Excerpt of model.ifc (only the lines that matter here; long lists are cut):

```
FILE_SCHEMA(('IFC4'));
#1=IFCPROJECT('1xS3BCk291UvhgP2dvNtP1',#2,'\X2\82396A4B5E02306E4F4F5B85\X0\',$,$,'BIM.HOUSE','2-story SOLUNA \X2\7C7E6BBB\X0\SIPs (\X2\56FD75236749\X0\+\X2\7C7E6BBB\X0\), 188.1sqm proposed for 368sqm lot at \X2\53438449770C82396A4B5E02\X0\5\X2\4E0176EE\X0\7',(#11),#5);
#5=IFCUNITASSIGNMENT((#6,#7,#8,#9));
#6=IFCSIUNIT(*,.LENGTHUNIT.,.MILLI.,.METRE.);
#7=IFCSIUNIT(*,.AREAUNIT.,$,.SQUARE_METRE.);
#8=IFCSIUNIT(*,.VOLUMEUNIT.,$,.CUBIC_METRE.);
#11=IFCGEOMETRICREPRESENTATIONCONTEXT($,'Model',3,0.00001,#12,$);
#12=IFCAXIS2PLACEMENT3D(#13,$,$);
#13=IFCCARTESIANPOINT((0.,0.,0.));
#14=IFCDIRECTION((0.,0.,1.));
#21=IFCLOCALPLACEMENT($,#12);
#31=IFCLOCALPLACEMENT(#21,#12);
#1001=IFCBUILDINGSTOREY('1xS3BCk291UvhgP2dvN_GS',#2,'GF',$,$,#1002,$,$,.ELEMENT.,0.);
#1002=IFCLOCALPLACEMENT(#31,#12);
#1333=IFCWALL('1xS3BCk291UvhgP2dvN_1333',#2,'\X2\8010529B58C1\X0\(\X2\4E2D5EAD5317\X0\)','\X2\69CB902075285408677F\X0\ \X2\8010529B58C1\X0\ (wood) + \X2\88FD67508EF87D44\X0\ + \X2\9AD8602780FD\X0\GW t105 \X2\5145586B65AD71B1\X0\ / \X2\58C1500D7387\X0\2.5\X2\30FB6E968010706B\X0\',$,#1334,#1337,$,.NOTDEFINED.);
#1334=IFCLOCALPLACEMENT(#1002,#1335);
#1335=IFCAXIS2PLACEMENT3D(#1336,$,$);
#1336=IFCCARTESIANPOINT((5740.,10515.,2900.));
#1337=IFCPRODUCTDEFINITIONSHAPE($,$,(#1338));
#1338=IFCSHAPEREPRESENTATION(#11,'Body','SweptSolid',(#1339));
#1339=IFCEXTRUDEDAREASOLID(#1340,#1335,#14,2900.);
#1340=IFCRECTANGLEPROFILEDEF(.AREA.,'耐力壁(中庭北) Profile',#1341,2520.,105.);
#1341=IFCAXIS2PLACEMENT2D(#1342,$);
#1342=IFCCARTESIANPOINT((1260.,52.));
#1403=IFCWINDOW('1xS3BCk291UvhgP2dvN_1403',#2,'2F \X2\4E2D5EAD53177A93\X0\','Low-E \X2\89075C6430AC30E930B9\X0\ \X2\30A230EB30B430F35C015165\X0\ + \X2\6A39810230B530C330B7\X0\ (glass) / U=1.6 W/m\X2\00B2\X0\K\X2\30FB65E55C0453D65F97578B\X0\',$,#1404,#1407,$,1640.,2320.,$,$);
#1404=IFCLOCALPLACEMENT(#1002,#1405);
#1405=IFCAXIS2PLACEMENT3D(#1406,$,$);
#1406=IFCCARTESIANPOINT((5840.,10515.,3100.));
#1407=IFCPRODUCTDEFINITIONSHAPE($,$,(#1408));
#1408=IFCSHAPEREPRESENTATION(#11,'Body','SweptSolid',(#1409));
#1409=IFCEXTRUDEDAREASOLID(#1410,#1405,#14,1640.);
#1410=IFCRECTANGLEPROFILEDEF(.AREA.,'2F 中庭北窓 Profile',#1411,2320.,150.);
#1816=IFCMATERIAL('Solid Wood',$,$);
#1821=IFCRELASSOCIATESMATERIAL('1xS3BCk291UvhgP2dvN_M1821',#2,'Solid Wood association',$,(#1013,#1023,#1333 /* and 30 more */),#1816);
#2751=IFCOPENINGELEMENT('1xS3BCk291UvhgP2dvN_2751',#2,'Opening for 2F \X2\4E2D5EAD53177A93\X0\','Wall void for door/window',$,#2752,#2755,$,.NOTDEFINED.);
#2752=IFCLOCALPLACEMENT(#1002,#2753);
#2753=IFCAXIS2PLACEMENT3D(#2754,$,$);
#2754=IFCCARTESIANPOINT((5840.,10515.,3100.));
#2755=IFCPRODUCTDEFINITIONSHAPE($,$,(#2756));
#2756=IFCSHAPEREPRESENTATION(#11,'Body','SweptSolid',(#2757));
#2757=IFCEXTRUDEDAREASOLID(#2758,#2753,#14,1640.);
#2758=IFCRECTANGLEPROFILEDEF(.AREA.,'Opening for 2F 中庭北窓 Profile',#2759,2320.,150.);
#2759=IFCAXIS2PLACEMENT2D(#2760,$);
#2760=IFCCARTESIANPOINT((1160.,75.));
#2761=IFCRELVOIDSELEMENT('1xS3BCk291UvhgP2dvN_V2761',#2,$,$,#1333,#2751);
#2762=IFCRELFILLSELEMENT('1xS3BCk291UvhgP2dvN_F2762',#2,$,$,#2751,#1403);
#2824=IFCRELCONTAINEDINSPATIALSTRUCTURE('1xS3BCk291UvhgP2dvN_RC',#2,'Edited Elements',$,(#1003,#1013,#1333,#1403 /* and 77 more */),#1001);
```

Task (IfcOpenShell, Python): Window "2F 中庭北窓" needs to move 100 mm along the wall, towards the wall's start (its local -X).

```python
import ifcopenshell
import ifcopenshell.api.geometry
import ifcopenshell.util.placement

model = ifcopenshell.open("model.ifc")

window = model.by_id(1403)
opening = window.FillsVoids[0].RelatingOpeningElement
wall = opening.VoidsElements[0].RelatingBuildingElement

wall_matrix = ifcopenshell.util.placement.get_local_placement(wall.ObjectPlacement)
shift = wall_matrix[:3, 0] * -100.0
before = ifcopenshell.util.placement.get_local_placement(window.ObjectPlacement)[:3, 3].copy()

# The window is not placed relative to its opening, so move both.
for product in (opening, window):
    matrix = ifcopenshell.util.placement.get_local_placement(product.ObjectPlacement)
    matrix[:3, 3] += shift
    ifcopenshell.api.geometry.edit_object_placement(model, product=product, matrix=matrix, is_si=False)

after = ifcopenshell.util.placement.get_local_placement(window.ObjectPlacement)[:3, 3]
print("window moved by", (after - before).round(3) + 0.0)

model.write("model_v2.ifc")
```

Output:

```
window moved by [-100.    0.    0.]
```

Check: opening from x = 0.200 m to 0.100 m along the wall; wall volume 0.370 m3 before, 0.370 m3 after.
